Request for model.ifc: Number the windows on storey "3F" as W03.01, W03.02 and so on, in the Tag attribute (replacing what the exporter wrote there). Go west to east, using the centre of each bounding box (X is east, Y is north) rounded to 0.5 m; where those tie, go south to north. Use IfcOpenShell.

First a look at what the model holds.

```python
import ifcopenshell
import ifcopenshell.util.element
import ifcopenshell.util.placement

model = ifcopenshell.open("model.ifc")
print(model.schema)
storey = next(s for s in model.by_type("IfcBuildingStorey") if s.Name == "3F")
windows = [e for e in ifcopenshell.util.element.get_decomposition(storey) if e.is_a("IfcWindow")]
for e in sorted(windows, key=lambda e: e.id()):
    origin = ifcopenshell.util.placement.get_local_placement(e.ObjectPlacement)[:3, 3]
    print(e.id(), e.Tag, e.Name, origin.round(2) + 0.0, sep=" | ")
```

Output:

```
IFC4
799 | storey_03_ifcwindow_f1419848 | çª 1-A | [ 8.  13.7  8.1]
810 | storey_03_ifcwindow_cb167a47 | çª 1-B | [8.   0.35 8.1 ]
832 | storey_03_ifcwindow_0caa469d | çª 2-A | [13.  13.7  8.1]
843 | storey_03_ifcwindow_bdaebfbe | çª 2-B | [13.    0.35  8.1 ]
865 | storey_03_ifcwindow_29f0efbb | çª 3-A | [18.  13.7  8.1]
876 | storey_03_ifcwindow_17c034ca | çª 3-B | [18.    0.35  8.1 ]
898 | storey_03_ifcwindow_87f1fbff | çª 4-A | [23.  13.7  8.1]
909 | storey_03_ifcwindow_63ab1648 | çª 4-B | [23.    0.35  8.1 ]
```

```python
import ifcopenshell
import ifcopenshell.geom
import ifcopenshell.util.element
import ifcopenshell.util.shape

model = ifcopenshell.open("model.ifc")
settings = ifcopenshell.geom.settings()
settings.set("use-world-coords", True)


def centre(element):
    shape = ifcopenshell.geom.create_shape(settings, element)
    return ifcopenshell.util.shape.get_bbox_centroid(shape.geometry)


storey = next(s for s in model.by_type("IfcBuildingStorey") if s.Name == "3F")
windows = [e for e in ifcopenshell.util.element.get_decomposition(storey) if e.is_a("IfcWindow")]

# Insertion points can sit at a corner or the storey origin, so sort by the geometry (in metres).
centres = {e: centre(e) for e in windows}
windows.sort(key=lambda e: (round(centres[e][0] / 0.5), centres[e][1]))

for i, e in enumerate(windows, start=1):
    number = f"W03.{i:02d}"
    e.Tag = number
    print(e.id(), number)

model.write("model_rev.ifc")
```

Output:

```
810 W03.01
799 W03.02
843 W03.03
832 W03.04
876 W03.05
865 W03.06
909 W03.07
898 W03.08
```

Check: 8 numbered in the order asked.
